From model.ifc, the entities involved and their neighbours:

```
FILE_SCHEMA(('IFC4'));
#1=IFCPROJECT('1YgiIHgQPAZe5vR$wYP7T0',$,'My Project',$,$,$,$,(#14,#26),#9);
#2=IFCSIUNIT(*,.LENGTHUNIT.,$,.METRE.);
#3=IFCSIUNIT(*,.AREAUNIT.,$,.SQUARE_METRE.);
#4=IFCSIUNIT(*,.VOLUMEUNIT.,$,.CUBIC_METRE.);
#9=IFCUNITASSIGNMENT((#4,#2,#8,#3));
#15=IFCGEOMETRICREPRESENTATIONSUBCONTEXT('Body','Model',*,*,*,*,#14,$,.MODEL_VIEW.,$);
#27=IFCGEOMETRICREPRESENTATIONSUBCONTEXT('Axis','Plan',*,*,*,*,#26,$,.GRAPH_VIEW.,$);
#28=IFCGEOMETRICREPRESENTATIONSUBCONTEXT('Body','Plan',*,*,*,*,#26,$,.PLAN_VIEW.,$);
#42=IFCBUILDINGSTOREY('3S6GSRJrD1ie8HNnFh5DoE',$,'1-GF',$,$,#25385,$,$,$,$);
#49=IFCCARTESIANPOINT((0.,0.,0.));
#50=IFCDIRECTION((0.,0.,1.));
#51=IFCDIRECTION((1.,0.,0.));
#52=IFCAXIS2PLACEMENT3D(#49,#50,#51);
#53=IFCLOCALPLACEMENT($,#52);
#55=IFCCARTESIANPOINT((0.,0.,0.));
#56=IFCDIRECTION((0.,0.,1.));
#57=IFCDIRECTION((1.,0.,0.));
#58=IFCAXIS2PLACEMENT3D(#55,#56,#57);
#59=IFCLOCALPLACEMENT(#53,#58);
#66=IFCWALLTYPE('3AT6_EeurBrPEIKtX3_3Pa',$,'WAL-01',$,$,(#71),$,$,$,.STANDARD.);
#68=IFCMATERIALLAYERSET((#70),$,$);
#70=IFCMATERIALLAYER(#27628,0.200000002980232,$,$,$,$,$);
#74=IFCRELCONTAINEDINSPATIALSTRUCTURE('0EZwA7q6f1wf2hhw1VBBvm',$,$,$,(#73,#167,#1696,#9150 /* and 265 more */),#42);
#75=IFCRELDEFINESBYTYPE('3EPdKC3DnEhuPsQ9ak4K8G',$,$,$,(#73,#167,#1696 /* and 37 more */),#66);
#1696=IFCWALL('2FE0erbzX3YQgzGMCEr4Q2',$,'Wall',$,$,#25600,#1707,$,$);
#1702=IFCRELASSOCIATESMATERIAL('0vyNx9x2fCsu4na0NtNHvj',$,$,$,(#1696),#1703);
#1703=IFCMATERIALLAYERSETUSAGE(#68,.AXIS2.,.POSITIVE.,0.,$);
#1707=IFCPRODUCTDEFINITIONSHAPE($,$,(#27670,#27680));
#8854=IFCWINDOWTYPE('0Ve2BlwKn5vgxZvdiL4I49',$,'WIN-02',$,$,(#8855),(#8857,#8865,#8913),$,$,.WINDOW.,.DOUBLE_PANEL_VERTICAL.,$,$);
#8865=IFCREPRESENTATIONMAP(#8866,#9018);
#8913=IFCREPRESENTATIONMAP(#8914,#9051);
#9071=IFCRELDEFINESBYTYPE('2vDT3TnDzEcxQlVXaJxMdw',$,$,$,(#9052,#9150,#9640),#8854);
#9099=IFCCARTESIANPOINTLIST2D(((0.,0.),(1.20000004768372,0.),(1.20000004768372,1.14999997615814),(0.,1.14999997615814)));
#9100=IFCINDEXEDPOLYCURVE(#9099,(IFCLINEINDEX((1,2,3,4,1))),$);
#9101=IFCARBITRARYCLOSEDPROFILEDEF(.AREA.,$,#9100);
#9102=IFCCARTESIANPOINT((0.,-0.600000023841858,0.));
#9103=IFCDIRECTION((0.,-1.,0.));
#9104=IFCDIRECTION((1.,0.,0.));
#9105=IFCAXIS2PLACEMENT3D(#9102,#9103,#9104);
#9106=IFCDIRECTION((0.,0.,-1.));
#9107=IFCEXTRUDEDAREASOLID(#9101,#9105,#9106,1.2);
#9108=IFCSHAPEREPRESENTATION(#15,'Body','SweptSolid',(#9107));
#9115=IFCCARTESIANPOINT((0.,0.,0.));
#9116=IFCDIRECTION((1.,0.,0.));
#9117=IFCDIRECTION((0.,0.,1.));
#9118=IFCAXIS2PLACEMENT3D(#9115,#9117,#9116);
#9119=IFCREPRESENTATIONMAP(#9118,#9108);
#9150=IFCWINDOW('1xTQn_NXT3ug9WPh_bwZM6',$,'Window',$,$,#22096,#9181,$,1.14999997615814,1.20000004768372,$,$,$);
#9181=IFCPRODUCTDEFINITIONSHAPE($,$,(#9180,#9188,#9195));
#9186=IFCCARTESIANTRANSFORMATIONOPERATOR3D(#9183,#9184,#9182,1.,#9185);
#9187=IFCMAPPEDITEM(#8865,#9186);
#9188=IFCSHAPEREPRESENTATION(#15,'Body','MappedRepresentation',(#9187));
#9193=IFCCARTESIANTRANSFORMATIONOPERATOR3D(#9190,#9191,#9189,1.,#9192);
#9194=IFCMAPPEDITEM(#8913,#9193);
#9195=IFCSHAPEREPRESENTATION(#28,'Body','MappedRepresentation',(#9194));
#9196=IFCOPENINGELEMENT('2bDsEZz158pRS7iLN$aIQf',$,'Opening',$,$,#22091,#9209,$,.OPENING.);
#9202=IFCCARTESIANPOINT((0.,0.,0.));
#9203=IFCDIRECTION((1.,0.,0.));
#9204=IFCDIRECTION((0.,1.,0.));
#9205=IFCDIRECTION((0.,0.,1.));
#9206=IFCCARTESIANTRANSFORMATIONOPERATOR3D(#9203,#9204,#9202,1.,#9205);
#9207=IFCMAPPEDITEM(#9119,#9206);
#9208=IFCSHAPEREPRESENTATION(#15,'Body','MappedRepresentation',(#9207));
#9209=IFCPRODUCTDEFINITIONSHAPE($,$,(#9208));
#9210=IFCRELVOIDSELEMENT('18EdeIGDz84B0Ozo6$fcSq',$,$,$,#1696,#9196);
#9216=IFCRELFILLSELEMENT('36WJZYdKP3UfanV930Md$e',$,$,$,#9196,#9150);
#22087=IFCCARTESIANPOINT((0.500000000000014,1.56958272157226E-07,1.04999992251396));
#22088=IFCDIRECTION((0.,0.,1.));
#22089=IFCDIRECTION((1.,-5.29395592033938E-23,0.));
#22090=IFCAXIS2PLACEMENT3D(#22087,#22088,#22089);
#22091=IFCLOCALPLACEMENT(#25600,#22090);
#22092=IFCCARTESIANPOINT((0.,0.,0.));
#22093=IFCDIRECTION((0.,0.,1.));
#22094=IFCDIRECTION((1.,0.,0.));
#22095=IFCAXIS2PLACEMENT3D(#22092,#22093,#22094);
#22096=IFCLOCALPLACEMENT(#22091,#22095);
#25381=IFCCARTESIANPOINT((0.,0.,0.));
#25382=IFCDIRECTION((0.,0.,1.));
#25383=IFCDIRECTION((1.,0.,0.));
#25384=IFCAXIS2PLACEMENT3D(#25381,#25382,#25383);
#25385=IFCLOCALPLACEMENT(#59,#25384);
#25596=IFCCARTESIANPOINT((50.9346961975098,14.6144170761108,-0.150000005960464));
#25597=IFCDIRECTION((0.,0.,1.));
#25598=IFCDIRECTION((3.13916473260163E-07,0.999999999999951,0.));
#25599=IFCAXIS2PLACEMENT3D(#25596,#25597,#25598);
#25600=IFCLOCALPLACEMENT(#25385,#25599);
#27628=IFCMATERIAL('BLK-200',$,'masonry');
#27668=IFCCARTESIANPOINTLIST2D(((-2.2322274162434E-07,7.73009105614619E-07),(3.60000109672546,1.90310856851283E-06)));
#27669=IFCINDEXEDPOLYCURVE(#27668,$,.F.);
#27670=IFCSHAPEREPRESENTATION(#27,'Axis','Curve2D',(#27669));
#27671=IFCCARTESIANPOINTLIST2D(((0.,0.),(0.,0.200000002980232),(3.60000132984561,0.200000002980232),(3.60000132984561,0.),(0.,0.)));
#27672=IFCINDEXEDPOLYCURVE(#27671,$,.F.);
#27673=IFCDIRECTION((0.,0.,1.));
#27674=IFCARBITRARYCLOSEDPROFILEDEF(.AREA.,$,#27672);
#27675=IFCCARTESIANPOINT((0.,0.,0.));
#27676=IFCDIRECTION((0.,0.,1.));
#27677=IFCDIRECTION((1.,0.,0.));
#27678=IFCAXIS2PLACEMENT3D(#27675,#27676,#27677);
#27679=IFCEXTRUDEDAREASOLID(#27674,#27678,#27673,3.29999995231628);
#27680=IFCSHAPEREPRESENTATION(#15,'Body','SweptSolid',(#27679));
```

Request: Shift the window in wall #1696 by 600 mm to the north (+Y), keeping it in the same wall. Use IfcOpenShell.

```python
import ifcopenshell
import ifcopenshell.api.geometry
import ifcopenshell.util.placement
import ifcopenshell.util.unit

model = ifcopenshell.open("model.ifc")
unit_scale = ifcopenshell.util.unit.calculate_unit_scale(model)

window = model.by_guid("1xTQn_NXT3ug9WPh_bwZM6")
opening = window.FillsVoids[0].RelatingOpeningElement
wall = opening.VoidsElements[0].RelatingBuildingElement

wall_matrix = ifcopenshell.util.placement.get_local_placement(wall.ObjectPlacement)
shift = wall_matrix[:3, 0] * 0.6 / unit_scale
before = ifcopenshell.util.placement.get_local_placement(window.ObjectPlacement)[:3, 3].copy()

# The window is placed relative to its opening, so it follows when the opening moves.
matrix = ifcopenshell.util.placement.get_local_placement(opening.ObjectPlacement)
matrix[:3, 3] += shift
ifcopenshell.api.geometry.edit_object_placement(
    model, product=opening, matrix=matrix, is_si=False, should_transform_children=True
)

after = ifcopenshell.util.placement.get_local_placement(window.ObjectPlacement)[:3, 3]
print("window moved by", (after - before).round(3) + 0.0)

model.write("model_edited.ifc")
```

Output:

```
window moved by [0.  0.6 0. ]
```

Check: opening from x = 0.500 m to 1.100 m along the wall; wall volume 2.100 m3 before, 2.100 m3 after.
